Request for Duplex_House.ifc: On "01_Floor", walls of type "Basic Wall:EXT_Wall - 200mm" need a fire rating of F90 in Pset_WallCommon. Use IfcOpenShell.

First a look at what the model holds.

```python
import ifcopenshell
import ifcopenshell.util.element

model = ifcopenshell.open("Duplex_House.ifc")
print(model.schema)
storey = next(s for s in model.by_type("IfcBuildingStorey") if s.Name == "01_Floor")
walls = [e for e in ifcopenshell.util.element.get_decomposition(storey) if e.is_a("IfcWall")]
seen = {}
for e in walls:
    element_type = ifcopenshell.util.element.get_type(e)
    key = (element_type.Name if element_type != e and element_type else None, ifcopenshell.util.element.get_pset(e, "Pset_WallCommon", "FireRating"))
    seen[key] = seen.get(key, 0) + 1
for (name, value), count in sorted(seen.items(), key=str):
    print(count, "x", name, "|", value)
```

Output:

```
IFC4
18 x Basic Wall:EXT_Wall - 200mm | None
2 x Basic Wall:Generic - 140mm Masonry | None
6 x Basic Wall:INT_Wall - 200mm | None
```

```python
import ifcopenshell
import ifcopenshell.api.pset
import ifcopenshell.util.element

model = ifcopenshell.open("Duplex_House.ifc")

storey = next(s for s in model.by_type("IfcBuildingStorey") if s.Name == "01_Floor")
walls = [e for e in ifcopenshell.util.element.get_decomposition(storey) if e.is_a("IfcWall")]

count = 0
for e in walls:
    element_type = ifcopenshell.util.element.get_type(e)
    if element_type in (None, e) or element_type.Name != "Basic Wall:EXT_Wall - 200mm":
        continue
    # add_pset returns the element's existing set when there is one.
    pset = ifcopenshell.api.pset.add_pset(model, product=e, name="Pset_WallCommon")
    ifcopenshell.api.pset.edit_pset(model, pset=pset, properties={"FireRating": "F90"})
    count += 1

print(count, "walls updated")

model.write("Duplex_House_v2.ifc")
```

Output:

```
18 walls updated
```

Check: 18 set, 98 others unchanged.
